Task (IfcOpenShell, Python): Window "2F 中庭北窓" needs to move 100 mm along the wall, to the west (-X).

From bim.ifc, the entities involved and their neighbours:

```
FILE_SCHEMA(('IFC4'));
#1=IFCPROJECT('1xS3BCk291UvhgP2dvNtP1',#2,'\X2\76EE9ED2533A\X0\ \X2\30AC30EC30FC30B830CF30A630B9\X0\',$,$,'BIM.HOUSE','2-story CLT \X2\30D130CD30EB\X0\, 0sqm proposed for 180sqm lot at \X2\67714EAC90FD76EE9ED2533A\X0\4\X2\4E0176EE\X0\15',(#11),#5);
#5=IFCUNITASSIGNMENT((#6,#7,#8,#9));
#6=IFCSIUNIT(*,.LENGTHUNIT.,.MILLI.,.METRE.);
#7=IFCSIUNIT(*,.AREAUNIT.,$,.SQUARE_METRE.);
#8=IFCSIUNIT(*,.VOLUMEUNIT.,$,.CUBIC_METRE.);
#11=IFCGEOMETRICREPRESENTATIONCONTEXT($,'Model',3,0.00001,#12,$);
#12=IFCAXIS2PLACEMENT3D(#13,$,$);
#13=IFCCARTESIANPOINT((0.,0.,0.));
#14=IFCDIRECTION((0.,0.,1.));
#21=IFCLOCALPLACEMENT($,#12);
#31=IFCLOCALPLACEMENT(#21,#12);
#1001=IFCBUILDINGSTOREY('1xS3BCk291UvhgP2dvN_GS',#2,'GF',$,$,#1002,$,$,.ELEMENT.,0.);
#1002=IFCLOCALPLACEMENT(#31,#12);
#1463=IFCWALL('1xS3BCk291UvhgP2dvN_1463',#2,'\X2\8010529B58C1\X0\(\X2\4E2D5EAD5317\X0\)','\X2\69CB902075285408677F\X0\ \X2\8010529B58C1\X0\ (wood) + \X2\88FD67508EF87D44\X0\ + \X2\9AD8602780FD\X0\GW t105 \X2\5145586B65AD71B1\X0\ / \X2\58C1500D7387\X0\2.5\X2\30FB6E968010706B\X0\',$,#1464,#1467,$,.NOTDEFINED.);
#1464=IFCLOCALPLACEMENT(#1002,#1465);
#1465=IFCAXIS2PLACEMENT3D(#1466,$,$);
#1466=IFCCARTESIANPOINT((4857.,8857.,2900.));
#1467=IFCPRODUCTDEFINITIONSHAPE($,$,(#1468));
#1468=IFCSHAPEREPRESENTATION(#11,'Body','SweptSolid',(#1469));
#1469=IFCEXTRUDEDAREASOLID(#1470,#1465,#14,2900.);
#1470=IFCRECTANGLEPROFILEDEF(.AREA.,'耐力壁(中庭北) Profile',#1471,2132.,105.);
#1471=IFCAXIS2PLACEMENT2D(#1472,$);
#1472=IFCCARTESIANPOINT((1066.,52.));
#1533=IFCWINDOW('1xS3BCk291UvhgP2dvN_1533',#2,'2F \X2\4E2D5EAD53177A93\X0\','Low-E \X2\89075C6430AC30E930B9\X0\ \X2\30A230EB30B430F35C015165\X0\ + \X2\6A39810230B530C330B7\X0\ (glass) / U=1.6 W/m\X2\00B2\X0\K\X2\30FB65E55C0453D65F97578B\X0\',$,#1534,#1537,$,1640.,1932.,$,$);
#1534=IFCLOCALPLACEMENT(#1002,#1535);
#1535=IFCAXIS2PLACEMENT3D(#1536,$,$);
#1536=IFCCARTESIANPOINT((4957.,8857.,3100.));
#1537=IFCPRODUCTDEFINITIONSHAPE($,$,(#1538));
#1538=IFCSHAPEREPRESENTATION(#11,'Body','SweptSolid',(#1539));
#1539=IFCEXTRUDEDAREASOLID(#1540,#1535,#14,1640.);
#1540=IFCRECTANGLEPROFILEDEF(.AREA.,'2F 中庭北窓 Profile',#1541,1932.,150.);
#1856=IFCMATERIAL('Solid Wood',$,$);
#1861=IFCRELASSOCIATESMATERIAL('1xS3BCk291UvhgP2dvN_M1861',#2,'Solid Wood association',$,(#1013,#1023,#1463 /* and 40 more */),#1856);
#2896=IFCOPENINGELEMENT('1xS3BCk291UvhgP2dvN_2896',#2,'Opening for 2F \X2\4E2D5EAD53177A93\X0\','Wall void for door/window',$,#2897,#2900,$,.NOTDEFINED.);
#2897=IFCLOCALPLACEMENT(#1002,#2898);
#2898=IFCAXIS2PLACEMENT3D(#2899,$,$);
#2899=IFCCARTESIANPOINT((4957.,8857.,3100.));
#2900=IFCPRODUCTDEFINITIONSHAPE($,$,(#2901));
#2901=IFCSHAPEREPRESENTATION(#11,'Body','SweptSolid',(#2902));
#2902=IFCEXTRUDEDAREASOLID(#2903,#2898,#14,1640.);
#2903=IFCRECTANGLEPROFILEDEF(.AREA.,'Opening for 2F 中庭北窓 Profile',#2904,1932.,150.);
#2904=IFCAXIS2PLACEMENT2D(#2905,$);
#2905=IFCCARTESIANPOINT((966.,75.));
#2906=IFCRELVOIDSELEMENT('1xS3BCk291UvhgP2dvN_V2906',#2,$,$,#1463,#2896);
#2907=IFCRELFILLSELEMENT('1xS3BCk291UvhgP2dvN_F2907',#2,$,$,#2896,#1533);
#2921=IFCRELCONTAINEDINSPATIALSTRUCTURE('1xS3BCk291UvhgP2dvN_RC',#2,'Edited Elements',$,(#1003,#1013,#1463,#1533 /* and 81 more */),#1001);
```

```python
import ifcopenshell
import ifcopenshell.api.geometry
import ifcopenshell.util.placement

model = ifcopenshell.open("bim.ifc")

window = model.by_id(1533)
opening = window.FillsVoids[0].RelatingOpeningElement
wall = opening.VoidsElements[0].RelatingBuildingElement

wall_matrix = ifcopenshell.util.placement.get_local_placement(wall.ObjectPlacement)
shift = wall_matrix[:3, 0] * -100.0
before = ifcopenshell.util.placement.get_local_placement(window.ObjectPlacement)[:3, 3].copy()

# The window is not placed relative to its opening, so move both.
for product in (opening, window):
    matrix = ifcopenshell.util.placement.get_local_placement(product.ObjectPlacement)
    matrix[:3, 3] += shift
    ifcopenshell.api.geometry.edit_object_placement(model, product=product, matrix=matrix, is_si=False)

after = ifcopenshell.util.placement.get_local_placement(window.ObjectPlacement)[:3, 3]
print("window moved by", (after - before).round(3) + 0.0)

model.write("bim_edited.ifc")
```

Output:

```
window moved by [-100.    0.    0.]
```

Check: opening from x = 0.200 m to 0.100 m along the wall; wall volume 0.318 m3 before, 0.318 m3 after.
